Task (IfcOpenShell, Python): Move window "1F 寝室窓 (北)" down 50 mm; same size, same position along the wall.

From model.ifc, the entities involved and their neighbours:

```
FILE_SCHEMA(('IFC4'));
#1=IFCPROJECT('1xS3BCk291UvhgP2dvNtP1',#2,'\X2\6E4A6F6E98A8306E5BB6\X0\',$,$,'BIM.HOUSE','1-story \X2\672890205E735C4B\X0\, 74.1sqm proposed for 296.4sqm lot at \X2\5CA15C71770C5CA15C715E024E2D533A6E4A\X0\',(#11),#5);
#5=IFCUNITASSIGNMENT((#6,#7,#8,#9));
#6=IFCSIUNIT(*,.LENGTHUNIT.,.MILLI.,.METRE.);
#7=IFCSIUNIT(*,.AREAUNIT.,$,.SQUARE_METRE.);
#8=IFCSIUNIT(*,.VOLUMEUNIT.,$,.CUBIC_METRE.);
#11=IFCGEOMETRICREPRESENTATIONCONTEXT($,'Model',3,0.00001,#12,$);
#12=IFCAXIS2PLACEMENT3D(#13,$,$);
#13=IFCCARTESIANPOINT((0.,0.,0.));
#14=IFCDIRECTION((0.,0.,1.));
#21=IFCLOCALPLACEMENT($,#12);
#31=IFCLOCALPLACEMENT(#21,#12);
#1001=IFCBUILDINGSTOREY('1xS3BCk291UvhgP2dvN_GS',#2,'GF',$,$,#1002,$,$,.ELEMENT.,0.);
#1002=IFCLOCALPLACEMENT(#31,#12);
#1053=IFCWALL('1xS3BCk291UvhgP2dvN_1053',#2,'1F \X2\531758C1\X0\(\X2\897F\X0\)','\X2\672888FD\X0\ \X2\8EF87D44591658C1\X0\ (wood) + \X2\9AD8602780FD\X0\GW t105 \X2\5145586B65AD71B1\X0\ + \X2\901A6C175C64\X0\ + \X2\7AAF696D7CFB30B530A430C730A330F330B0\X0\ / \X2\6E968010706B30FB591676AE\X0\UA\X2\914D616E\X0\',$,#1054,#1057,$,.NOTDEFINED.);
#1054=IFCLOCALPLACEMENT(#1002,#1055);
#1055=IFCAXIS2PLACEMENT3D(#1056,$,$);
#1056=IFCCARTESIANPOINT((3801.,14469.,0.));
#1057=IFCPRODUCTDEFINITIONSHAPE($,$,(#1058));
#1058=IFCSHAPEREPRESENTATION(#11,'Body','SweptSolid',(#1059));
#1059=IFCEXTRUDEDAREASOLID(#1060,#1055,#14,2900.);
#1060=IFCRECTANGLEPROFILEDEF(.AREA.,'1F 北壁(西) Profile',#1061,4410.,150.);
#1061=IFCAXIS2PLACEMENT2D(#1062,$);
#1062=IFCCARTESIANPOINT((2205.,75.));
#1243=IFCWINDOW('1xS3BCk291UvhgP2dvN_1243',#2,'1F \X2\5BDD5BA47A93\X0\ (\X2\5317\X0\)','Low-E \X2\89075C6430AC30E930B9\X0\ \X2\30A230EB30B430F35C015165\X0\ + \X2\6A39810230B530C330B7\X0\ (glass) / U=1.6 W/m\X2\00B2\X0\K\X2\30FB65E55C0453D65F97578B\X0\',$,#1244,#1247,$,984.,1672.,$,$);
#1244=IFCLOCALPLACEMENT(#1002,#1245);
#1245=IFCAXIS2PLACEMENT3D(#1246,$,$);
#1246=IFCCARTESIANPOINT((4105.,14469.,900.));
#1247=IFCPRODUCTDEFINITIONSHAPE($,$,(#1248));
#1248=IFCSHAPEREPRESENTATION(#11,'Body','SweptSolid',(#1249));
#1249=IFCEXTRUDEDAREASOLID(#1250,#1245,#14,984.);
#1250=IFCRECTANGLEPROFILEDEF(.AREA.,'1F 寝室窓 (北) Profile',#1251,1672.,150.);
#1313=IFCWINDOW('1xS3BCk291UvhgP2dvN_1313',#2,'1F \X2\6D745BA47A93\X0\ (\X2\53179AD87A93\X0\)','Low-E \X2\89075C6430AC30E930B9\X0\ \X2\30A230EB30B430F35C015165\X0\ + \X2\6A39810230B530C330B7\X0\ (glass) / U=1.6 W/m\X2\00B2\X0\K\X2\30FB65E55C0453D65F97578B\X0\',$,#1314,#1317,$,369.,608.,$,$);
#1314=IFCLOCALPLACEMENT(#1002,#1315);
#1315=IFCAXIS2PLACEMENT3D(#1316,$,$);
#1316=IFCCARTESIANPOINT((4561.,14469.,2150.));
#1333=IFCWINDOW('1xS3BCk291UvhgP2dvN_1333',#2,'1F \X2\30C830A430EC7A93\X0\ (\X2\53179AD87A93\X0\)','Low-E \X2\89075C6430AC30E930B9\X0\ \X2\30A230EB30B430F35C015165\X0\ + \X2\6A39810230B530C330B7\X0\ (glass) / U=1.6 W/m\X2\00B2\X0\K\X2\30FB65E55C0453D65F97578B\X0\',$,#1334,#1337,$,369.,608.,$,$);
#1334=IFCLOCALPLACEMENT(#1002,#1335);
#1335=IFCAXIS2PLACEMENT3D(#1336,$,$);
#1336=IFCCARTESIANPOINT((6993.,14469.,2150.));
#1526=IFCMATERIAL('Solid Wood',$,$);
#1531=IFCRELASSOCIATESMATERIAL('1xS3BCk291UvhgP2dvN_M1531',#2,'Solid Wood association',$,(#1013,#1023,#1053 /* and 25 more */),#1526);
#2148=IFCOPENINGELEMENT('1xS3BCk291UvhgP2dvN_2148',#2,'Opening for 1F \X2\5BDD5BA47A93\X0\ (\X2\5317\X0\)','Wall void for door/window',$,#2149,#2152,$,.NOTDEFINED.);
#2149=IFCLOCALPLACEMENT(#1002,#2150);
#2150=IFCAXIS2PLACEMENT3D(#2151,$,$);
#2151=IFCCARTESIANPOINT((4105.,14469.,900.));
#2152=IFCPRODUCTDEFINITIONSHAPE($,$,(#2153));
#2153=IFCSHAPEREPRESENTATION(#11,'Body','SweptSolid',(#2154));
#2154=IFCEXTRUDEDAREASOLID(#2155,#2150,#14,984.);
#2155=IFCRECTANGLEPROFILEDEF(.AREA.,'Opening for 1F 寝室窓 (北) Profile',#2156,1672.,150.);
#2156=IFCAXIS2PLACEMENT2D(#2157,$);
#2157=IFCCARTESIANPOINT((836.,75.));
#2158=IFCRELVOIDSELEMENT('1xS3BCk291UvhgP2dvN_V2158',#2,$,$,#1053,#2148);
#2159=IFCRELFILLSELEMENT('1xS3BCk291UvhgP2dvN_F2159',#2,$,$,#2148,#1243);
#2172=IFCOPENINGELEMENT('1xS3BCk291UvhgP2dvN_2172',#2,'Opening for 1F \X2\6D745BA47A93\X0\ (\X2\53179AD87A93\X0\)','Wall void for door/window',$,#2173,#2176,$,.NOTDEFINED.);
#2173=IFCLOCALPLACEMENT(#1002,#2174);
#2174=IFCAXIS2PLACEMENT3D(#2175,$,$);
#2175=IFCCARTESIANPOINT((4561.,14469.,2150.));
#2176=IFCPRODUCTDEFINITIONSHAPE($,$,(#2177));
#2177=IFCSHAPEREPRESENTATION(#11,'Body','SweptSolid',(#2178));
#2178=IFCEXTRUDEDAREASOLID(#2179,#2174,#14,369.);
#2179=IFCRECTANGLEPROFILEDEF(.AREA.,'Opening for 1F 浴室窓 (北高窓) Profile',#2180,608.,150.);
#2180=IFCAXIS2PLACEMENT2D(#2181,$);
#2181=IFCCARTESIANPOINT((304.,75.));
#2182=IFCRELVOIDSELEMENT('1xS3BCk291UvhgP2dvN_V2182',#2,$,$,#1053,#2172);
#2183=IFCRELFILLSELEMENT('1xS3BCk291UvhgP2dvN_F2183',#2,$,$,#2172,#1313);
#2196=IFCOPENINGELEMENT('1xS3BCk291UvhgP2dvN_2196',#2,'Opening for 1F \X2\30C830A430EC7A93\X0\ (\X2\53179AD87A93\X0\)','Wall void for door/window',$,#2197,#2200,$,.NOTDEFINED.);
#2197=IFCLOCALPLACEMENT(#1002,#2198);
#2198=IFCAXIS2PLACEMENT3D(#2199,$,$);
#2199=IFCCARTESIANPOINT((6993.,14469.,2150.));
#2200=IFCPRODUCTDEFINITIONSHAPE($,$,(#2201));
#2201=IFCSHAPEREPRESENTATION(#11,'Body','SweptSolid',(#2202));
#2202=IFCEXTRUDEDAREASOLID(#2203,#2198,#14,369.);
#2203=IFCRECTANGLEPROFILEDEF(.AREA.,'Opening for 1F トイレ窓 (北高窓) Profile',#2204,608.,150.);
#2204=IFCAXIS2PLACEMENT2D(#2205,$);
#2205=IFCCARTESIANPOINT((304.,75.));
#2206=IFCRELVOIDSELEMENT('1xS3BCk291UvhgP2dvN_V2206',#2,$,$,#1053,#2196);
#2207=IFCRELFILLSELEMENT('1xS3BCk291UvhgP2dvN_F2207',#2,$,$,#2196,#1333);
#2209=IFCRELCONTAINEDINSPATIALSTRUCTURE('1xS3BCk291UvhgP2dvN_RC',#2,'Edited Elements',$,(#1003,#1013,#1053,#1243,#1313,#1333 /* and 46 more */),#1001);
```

```python
import numpy as np
import ifcopenshell
import ifcopenshell.api.geometry
import ifcopenshell.util.placement
import ifcopenshell.util.unit

model = ifcopenshell.open("model.ifc")
unit_scale = ifcopenshell.util.unit.calculate_unit_scale(model)

window = model.by_guid("1xS3BCk291UvhgP2dvN_1243")
opening = window.FillsVoids[0].RelatingOpeningElement
dz = -50.0

shift = np.array([0.0, 0.0, dz])
# The window is not placed relative to its opening, so move both.
for product in (opening, window):
    matrix = ifcopenshell.util.placement.get_local_placement(product.ObjectPlacement)
    matrix[:3, 3] += shift
    ifcopenshell.api.geometry.edit_object_placement(model, product=product, matrix=matrix, is_si=False)

print(f"moved by {dz * unit_scale:+.3f} m")

model.write("model_v2.ifc")
```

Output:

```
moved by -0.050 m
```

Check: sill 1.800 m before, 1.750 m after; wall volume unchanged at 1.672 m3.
